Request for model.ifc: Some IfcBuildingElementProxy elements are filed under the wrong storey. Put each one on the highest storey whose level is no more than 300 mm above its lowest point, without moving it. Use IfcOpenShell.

First a look at what the model holds.

```python
import ifcopenshell
import ifcopenshell.util.element
import ifcopenshell.util.placement

model = ifcopenshell.open("model.ifc")
print(model.schema)
for storey in model.by_type("IfcBuildingStorey"):
    level = ifcopenshell.util.placement.get_storey_elevation(storey)
    count = sum(e.is_a("IfcBuildingElementProxy") for e in ifcopenshell.util.element.get_contained(storey))
    print(storey.id(), storey.Name, round(level, 3), count, sep=" | ")
```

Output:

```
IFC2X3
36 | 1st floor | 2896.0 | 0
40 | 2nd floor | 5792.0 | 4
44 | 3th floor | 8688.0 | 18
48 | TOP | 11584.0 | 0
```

```python
import ifcopenshell
import ifcopenshell.api.spatial
import ifcopenshell.geom
import ifcopenshell.util.element
import ifcopenshell.util.placement
import ifcopenshell.util.shape
import ifcopenshell.util.unit

model = ifcopenshell.open("model.ifc")
unit_scale = ifcopenshell.util.unit.calculate_unit_scale(model)
settings = ifcopenshell.geom.settings()

levels = sorted(
    ((ifcopenshell.util.placement.get_storey_elevation(s) * unit_scale, s) for s in model.by_type("IfcBuildingStorey")),
    key=lambda pair: pair[0],
)

for e in model.by_type("IfcBuildingElementProxy"):
    current = e.ContainedInStructure[0].RelatingStructure if e.ContainedInStructure else None
    if current is None or not current.is_a("IfcBuildingStorey"):
        continue
    shape = ifcopenshell.geom.create_shape(settings, e)
    bottom = ifcopenshell.util.shape.get_shape_bottom_elevation(shape, shape.geometry)
    below = [s for level, s in levels if level <= bottom + 0.3]
    storey = below[-1] if below else levels[0][1]
    if storey != current:
        # assign_container keeps the world position.
        ifcopenshell.api.spatial.assign_container(model, products=[e], relating_structure=storey)
        print(e.id(), current.Name, "->", storey.Name)

model.write("model_edited.ifc")
```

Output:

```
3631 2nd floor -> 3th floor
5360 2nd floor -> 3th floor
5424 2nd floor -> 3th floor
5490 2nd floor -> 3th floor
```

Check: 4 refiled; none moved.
